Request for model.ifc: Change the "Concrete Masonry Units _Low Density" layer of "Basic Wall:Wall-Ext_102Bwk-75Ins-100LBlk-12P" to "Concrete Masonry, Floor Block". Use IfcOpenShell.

First a look at what the model holds.

```python
import ifcopenshell
import ifcopenshell.util.element

model = ifcopenshell.open("model.ifc")
print(model.schema)
for layer_set in model.by_type("IfcMaterialLayerSet"):
    if layer_set.LayerSetName == "Basic Wall:Wall-Ext_102Bwk-75Ins-100LBlk-12P":
        for layer in layer_set.MaterialLayers:
            print(layer.id(), layer.Material and layer.Material.Name, layer.LayerThickness, sep=" | ")
        print(len(ifcopenshell.util.element.get_elements_by_material(model, layer_set)), "elements and types use it")
print(sorted(m.Name for m in model.by_type("IfcMaterial") if m.Name)[:60])
```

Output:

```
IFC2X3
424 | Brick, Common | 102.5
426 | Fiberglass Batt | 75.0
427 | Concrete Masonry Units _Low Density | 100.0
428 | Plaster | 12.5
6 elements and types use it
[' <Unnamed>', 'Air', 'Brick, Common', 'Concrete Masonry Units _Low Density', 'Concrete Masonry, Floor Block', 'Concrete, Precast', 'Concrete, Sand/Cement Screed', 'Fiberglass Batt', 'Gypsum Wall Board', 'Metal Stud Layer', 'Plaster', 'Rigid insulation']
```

```python
import ifcopenshell
import ifcopenshell.api.material

model = ifcopenshell.open("model.ifc")

layer_set = next(s for s in model.by_type("IfcMaterialLayerSet") if s.LayerSetName == "Basic Wall:Wall-Ext_102Bwk-75Ins-100LBlk-12P")
layer = next(l for l in layer_set.MaterialLayers if l.Material and l.Material.Name == "Concrete Masonry Units _Low Density")
material = next(m for m in model.by_type("IfcMaterial") if m.Name == "Concrete Masonry, Floor Block")

# Point this one layer at the other material; renaming the old one would change it everywhere.
ifcopenshell.api.material.edit_layer(model, layer=layer, attributes={}, material=material)

print([l.Material.Name if l.Material else None for l in layer_set.MaterialLayers])

model.write("model_v2.ifc")
```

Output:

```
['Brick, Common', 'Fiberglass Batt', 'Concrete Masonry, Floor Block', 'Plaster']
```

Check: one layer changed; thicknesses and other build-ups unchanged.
